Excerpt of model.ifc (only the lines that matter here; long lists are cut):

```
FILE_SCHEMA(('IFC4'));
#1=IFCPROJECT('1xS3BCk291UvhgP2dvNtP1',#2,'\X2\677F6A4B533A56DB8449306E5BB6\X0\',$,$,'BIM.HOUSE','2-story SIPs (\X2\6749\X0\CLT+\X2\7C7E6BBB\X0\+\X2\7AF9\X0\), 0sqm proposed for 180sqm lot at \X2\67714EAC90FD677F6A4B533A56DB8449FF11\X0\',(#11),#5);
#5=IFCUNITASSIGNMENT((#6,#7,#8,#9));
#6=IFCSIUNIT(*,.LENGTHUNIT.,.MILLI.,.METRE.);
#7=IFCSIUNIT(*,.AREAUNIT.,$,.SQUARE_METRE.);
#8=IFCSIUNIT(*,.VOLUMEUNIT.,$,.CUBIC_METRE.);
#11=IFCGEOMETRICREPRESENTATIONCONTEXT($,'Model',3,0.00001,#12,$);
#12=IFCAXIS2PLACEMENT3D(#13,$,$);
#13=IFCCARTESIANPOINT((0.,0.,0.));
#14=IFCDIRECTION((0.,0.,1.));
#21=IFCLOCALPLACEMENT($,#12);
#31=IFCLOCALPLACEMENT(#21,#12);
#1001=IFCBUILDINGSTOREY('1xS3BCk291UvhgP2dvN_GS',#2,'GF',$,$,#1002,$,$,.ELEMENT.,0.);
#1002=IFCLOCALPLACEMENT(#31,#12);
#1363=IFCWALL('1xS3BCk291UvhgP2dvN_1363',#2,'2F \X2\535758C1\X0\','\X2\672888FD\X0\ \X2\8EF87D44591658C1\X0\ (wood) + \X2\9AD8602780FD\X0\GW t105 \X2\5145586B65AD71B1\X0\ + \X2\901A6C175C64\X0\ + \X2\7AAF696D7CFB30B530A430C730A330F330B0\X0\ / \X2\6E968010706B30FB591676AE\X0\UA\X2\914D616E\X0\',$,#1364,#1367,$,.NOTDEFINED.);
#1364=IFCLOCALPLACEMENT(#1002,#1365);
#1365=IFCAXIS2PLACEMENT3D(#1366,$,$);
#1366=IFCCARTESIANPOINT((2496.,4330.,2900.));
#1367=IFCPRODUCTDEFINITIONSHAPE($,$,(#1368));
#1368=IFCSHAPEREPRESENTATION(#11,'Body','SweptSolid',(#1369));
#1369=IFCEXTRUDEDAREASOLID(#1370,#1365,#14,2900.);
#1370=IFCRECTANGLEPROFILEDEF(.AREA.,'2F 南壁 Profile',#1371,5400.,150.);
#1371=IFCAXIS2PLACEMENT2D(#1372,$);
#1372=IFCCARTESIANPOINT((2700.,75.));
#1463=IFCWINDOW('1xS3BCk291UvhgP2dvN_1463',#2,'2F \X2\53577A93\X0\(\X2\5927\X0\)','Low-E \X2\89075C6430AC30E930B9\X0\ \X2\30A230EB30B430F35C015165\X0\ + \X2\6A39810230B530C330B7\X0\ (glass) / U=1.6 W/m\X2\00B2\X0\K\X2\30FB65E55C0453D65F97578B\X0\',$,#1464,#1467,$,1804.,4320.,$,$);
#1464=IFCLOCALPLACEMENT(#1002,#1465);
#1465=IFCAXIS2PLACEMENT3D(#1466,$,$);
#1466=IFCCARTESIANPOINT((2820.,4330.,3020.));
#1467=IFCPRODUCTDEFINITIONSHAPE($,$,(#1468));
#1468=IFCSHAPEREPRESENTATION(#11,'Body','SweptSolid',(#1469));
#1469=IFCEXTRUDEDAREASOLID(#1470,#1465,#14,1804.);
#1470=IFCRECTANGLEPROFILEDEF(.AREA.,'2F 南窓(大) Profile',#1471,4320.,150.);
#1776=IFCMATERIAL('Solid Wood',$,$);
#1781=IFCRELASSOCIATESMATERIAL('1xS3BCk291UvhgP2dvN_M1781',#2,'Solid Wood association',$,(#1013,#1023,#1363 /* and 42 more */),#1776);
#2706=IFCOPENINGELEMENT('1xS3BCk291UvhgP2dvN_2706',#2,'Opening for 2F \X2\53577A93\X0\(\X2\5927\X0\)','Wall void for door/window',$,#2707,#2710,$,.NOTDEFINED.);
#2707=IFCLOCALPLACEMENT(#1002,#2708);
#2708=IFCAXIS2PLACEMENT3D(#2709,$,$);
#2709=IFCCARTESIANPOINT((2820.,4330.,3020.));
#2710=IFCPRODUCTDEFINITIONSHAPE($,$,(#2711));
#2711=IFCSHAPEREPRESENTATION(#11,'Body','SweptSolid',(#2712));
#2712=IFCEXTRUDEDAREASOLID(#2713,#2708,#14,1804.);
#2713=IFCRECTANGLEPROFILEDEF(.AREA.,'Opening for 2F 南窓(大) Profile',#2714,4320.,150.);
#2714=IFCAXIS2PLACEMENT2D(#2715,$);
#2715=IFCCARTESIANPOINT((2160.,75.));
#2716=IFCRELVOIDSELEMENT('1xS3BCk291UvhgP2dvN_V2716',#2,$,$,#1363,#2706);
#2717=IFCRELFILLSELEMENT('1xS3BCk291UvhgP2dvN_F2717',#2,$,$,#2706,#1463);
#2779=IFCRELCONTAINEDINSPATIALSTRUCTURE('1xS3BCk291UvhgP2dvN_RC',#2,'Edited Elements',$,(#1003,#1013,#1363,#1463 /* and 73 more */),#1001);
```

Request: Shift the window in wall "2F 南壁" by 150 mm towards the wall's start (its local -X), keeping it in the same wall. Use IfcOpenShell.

```python
import ifcopenshell
import ifcopenshell.api.geometry
import ifcopenshell.util.placement
import ifcopenshell.util.unit

model = ifcopenshell.open("model.ifc")
unit_scale = ifcopenshell.util.unit.calculate_unit_scale(model)

window = model.by_id(1463)
opening = window.FillsVoids[0].RelatingOpeningElement
wall = opening.VoidsElements[0].RelatingBuildingElement

wall_matrix = ifcopenshell.util.placement.get_local_placement(wall.ObjectPlacement)
shift = wall_matrix[:3, 0] * -0.15 / unit_scale
before = ifcopenshell.util.placement.get_local_placement(window.ObjectPlacement)[:3, 3].copy()

# The window is not placed relative to its opening, so move both.
for product in (opening, window):
    matrix = ifcopenshell.util.placement.get_local_placement(product.ObjectPlacement)
    matrix[:3, 3] += shift
    ifcopenshell.api.geometry.edit_object_placement(model, product=product, matrix=matrix, is_si=False)

after = ifcopenshell.util.placement.get_local_placement(window.ObjectPlacement)[:3, 3]
print("window moved by", (after - before).round(3) + 0.0)

model.write("model_updated.ifc")
```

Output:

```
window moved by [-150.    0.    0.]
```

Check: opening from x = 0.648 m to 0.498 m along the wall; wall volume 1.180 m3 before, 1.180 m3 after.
